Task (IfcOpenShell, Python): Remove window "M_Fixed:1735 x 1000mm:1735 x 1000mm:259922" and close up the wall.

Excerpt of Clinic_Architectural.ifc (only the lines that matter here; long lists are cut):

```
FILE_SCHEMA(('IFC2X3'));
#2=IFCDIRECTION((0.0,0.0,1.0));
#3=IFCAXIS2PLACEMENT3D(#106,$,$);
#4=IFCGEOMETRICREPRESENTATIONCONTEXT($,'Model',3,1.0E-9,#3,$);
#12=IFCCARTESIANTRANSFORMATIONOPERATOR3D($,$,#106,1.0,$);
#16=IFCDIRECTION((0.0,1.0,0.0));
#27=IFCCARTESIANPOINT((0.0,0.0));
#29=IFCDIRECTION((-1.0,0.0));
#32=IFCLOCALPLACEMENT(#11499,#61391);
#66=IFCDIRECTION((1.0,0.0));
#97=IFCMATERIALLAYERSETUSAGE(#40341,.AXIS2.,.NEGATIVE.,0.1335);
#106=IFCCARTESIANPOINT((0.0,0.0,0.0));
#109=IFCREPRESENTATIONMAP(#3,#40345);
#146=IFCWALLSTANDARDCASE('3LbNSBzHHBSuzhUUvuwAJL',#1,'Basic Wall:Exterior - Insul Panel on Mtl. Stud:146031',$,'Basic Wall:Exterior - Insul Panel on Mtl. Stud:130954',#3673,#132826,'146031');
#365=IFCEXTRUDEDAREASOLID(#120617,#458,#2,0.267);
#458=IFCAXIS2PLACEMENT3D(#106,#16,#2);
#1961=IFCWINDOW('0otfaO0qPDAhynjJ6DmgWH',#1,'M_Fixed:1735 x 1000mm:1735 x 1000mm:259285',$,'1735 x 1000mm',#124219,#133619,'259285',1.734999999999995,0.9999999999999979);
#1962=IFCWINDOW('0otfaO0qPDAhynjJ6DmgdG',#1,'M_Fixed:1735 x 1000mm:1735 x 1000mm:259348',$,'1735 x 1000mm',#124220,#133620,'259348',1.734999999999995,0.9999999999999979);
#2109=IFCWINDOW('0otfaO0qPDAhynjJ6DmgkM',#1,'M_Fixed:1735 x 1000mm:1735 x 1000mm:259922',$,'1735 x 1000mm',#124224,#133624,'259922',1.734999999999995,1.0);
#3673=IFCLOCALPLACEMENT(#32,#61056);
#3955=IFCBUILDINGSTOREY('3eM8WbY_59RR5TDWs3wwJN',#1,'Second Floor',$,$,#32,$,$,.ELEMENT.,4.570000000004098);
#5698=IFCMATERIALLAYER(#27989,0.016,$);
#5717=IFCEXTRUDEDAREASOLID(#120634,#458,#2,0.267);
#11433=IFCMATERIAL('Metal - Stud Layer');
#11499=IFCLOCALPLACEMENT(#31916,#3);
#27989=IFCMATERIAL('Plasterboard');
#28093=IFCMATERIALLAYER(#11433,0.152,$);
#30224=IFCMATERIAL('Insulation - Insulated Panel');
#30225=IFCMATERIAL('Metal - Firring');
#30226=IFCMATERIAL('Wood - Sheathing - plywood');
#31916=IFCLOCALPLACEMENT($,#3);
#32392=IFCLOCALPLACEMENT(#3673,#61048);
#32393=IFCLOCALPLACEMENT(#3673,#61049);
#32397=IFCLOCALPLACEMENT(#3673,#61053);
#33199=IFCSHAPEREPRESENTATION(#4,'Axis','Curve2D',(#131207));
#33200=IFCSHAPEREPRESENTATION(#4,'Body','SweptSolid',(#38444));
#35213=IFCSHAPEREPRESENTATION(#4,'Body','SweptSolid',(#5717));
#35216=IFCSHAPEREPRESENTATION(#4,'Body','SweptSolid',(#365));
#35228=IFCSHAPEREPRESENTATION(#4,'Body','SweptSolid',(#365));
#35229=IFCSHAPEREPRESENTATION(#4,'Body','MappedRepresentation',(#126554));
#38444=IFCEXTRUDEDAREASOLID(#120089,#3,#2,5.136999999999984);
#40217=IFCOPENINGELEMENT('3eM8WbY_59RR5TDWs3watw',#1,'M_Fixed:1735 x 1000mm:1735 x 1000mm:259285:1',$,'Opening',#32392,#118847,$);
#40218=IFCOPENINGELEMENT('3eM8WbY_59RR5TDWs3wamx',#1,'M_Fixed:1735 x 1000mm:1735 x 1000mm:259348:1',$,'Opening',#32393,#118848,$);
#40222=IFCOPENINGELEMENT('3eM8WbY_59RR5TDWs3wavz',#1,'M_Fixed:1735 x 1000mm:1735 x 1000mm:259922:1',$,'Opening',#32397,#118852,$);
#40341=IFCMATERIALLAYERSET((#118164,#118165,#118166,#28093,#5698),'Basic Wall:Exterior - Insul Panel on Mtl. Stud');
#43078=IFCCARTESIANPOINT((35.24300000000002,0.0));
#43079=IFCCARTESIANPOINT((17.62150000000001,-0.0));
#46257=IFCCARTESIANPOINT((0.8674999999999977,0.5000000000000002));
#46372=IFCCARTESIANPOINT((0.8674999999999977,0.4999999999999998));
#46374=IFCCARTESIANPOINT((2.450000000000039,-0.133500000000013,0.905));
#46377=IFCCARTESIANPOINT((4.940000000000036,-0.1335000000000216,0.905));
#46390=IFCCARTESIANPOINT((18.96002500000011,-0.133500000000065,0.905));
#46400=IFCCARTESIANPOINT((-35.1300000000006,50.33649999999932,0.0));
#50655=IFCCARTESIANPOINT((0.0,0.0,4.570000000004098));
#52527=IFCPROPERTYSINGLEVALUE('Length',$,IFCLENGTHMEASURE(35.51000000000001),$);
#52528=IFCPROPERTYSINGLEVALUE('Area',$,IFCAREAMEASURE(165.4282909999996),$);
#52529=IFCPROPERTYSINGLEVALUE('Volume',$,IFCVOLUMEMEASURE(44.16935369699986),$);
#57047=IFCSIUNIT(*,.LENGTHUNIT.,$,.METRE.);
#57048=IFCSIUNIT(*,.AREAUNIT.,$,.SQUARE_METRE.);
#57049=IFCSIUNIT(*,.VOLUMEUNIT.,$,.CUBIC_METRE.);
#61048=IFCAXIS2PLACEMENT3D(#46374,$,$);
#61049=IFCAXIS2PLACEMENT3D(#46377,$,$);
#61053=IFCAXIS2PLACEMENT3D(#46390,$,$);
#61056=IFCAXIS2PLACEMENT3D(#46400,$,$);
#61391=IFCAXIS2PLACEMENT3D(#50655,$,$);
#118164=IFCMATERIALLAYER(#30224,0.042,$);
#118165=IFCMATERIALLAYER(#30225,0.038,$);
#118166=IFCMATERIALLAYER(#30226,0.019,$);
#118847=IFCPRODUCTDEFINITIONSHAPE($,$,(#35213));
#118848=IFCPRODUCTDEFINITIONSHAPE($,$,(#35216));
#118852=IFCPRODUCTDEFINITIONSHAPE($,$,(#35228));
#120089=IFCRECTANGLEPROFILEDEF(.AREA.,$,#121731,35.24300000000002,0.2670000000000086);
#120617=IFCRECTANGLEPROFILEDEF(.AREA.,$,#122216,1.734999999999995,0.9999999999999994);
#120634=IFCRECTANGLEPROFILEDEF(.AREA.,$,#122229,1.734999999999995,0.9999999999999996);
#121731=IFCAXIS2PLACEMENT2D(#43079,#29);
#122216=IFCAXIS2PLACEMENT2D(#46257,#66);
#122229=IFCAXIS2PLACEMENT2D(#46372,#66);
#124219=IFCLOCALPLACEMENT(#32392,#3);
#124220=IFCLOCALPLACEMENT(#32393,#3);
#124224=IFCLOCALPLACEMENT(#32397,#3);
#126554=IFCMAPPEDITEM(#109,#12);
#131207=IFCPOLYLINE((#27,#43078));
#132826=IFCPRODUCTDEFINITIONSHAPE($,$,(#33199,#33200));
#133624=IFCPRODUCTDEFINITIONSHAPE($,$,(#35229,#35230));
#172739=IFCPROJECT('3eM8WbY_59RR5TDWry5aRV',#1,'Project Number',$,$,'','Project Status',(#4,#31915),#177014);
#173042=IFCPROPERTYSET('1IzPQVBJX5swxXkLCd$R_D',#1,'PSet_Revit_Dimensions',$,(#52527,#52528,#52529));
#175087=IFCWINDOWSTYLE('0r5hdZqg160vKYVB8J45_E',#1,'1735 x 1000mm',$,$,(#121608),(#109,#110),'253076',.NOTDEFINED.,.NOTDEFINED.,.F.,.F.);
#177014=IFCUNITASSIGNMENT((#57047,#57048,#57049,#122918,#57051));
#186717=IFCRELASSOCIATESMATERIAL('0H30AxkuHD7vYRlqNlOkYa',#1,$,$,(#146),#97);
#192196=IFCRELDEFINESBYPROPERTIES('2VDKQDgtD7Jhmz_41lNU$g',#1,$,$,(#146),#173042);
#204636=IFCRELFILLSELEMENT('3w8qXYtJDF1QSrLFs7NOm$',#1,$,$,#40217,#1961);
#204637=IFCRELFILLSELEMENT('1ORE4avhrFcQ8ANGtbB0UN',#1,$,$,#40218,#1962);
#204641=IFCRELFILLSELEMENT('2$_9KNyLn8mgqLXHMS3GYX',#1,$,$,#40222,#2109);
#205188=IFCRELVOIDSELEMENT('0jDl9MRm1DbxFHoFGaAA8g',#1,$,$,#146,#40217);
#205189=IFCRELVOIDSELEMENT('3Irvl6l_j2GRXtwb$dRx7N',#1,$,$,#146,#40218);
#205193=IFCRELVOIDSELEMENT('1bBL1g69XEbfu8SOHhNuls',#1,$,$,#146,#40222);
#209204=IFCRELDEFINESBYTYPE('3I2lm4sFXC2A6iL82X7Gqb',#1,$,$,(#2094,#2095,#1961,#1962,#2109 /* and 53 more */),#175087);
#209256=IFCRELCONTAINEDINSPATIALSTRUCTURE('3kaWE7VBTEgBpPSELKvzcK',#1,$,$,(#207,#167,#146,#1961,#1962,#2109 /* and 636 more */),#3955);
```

```python
import ifcopenshell
import ifcopenshell.api.feature
import ifcopenshell.api.pset
import ifcopenshell.api.root
import ifcopenshell.geom
import ifcopenshell.util.element
import ifcopenshell.util.shape
import ifcopenshell.util.unit

model = ifcopenshell.open("Clinic_Architectural.ifc")
area_scale = ifcopenshell.util.unit.calculate_unit_scale(model, "AREAUNIT")
volume_scale = ifcopenshell.util.unit.calculate_unit_scale(model, "VOLUMEUNIT")
settings = ifcopenshell.geom.settings()


def volume(element):
    """Net volume in cubic metres, openings subtracted."""
    shape = ifcopenshell.geom.create_shape(settings, element)
    return ifcopenshell.util.shape.get_volume(shape.geometry)


window = model.by_guid("0otfaO0qPDAhynjJ6DmgkM")
opening = window.FillsVoids[0].RelatingOpeningElement
wall = opening.VoidsElements[0].RelatingBuildingElement
before = volume(wall)

ifcopenshell.api.root.remove_product(model, product=window)
ifcopenshell.api.feature.remove_feature(model, feature=opening)

after = volume(wall)
thickness = 0.267  # wall thickness in metres

# Update the wall's stored quantities.
pset = model.by_id(ifcopenshell.util.element.get_pset(wall, "PSet_Revit_Dimensions", should_inherit=False)["id"])
ifcopenshell.api.pset.edit_pset(model, pset=pset, properties={
    "Area": model.create_entity("IfcAreaMeasure", after / thickness / area_scale),
    "Volume": model.create_entity("IfcVolumeMeasure", after / volume_scale),
})

print(f"wall volume {before:.3f} -> {after:.3f} m3")

model.write("Clinic_Architectural_rev.ifc")
```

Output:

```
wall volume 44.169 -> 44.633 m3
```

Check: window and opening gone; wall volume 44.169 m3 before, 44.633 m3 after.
